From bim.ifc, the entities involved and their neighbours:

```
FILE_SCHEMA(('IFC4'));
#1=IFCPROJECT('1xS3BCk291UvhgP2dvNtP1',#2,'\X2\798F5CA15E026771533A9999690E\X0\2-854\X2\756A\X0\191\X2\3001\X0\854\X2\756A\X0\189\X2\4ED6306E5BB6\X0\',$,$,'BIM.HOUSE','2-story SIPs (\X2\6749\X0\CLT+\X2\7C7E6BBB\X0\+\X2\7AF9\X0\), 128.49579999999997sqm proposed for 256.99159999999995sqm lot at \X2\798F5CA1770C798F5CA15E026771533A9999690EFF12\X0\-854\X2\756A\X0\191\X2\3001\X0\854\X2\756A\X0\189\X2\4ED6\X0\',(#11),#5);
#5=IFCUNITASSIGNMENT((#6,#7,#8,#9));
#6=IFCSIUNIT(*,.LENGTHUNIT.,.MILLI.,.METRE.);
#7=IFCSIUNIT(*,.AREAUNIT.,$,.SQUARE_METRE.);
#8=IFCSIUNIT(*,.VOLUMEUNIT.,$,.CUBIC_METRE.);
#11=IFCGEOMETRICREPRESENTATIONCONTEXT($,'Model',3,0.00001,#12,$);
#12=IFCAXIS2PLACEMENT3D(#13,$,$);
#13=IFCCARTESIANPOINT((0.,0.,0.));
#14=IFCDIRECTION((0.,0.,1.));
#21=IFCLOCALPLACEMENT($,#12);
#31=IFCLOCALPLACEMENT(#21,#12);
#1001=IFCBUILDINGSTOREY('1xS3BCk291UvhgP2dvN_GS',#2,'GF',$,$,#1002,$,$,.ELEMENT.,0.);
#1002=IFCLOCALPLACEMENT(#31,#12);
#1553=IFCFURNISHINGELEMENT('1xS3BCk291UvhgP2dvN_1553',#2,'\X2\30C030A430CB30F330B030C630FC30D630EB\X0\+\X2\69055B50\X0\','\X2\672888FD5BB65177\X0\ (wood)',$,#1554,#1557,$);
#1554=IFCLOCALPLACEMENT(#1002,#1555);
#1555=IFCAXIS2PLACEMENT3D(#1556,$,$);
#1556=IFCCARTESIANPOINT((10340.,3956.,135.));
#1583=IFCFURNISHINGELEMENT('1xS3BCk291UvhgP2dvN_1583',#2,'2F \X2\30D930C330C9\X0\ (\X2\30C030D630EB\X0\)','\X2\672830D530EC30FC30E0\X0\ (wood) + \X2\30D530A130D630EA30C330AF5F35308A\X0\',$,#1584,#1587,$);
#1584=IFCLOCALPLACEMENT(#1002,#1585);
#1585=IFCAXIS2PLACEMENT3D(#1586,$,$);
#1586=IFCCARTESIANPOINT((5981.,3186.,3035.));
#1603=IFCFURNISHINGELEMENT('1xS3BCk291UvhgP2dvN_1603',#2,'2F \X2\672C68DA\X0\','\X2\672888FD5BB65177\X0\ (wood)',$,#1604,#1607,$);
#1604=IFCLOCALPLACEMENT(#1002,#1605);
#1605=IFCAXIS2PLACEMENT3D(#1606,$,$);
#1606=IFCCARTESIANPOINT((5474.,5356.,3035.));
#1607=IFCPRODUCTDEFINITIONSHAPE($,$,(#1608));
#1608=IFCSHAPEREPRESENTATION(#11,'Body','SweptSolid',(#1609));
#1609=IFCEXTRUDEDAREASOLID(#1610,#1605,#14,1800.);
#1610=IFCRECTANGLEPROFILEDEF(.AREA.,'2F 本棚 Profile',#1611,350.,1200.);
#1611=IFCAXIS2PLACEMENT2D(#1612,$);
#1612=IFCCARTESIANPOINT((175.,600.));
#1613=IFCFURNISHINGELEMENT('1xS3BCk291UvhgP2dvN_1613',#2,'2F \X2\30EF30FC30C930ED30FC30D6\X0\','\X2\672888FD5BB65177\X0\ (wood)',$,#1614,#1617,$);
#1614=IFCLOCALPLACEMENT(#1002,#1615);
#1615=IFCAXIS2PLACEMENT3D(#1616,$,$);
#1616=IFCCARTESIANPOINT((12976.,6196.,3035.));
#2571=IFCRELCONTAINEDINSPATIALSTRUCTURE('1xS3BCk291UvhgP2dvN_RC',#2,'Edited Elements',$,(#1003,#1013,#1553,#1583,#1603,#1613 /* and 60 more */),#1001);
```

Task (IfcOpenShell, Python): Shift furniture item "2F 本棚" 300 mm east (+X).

```python
import ifcopenshell
import ifcopenshell.api.geometry
import ifcopenshell.util.placement

model = ifcopenshell.open("bim.ifc")

item = model.by_id(1603)
matrix = ifcopenshell.util.placement.get_local_placement(item.ObjectPlacement)
matrix[0, 3] += 300.0
ifcopenshell.api.geometry.edit_object_placement(model, product=item, matrix=matrix, is_si=False)

print(ifcopenshell.util.placement.get_local_placement(item.ObjectPlacement).round(3) + 0.0)

model.write("bim-out.ifc")
```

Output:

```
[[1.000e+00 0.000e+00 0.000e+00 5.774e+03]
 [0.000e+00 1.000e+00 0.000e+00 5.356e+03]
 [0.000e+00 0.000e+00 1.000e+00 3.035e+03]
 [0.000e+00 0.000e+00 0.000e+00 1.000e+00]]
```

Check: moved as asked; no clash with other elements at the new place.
